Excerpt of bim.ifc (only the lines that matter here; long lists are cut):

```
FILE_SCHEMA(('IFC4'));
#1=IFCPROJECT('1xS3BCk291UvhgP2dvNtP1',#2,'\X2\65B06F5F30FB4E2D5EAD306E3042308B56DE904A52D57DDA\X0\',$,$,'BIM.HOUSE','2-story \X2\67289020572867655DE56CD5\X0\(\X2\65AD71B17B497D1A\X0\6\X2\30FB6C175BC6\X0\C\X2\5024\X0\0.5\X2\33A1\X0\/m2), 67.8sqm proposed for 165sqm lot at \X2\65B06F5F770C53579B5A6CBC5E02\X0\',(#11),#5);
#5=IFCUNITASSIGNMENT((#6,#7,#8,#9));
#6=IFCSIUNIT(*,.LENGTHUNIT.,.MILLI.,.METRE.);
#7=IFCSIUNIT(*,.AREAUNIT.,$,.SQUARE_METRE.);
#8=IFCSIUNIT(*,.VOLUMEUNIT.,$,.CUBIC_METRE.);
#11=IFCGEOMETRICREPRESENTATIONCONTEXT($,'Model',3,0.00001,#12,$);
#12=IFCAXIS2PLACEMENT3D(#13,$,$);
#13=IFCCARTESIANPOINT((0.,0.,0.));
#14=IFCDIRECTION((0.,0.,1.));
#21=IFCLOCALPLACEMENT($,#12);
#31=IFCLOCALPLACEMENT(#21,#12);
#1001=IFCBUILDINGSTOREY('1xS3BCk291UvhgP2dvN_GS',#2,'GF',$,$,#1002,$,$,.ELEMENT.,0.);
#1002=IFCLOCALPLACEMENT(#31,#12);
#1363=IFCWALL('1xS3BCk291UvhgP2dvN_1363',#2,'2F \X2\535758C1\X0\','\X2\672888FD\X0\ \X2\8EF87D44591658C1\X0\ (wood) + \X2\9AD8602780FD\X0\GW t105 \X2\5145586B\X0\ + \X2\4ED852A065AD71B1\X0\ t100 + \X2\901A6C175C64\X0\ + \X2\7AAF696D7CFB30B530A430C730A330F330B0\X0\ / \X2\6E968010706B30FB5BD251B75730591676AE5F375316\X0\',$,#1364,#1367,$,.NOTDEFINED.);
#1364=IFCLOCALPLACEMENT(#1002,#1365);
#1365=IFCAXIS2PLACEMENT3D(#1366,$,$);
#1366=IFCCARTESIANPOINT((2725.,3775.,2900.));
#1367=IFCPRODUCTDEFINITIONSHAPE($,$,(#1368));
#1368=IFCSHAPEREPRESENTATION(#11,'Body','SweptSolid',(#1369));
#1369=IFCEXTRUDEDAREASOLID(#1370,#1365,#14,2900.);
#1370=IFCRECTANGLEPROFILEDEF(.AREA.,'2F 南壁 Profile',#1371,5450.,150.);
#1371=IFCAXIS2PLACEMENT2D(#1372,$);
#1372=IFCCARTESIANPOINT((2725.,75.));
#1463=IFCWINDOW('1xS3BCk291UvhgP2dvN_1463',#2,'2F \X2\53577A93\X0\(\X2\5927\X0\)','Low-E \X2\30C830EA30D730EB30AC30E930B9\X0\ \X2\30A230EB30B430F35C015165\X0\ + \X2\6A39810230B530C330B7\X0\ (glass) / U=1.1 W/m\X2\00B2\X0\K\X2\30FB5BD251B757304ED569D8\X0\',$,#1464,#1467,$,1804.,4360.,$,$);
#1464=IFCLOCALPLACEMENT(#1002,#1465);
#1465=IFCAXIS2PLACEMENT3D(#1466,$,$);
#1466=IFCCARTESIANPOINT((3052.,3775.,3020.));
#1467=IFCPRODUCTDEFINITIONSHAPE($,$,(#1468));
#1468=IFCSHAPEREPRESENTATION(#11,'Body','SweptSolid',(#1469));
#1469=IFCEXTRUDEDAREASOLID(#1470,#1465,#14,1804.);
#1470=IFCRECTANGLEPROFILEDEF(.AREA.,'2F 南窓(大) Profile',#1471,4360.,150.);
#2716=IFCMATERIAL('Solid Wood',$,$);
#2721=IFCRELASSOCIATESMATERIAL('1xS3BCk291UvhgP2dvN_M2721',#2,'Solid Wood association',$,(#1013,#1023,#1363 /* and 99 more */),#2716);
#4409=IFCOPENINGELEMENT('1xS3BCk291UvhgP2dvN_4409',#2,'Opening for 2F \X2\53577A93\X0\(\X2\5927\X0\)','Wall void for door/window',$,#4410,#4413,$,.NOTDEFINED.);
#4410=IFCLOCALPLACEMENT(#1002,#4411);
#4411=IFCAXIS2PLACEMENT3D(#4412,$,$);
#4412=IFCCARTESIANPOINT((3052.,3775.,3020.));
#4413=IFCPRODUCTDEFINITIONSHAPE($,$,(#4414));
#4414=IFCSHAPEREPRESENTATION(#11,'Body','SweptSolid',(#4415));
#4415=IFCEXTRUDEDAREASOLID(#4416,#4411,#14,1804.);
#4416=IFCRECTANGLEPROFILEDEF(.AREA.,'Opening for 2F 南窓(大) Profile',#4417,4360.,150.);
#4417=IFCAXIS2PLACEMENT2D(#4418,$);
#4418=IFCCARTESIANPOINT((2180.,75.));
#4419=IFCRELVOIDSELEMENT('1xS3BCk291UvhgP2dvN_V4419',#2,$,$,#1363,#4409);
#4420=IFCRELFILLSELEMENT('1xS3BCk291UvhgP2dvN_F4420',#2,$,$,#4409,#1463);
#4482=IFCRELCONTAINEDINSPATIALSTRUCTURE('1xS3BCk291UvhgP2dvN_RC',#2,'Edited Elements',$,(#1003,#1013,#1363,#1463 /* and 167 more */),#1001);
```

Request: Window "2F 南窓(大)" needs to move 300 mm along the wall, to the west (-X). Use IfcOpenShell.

```python
import ifcopenshell
import ifcopenshell.api.geometry
import ifcopenshell.util.placement
import ifcopenshell.util.unit

model = ifcopenshell.open("bim.ifc")
unit_scale = ifcopenshell.util.unit.calculate_unit_scale(model)

window = model.by_id(1463)
opening = window.FillsVoids[0].RelatingOpeningElement
wall = opening.VoidsElements[0].RelatingBuildingElement

wall_matrix = ifcopenshell.util.placement.get_local_placement(wall.ObjectPlacement)
shift = wall_matrix[:3, 0] * -0.3 / unit_scale
before = ifcopenshell.util.placement.get_local_placement(window.ObjectPlacement)[:3, 3].copy()

# The window is not placed relative to its opening, so move both.
for product in (opening, window):
    matrix = ifcopenshell.util.placement.get_local_placement(product.ObjectPlacement)
    matrix[:3, 3] += shift
    ifcopenshell.api.geometry.edit_object_placement(model, product=product, matrix=matrix, is_si=False)

after = ifcopenshell.util.placement.get_local_placement(window.ObjectPlacement)[:3, 3]
print("window moved by", (after - before).round(3) + 0.0)

model.write("bim_v2.ifc")
```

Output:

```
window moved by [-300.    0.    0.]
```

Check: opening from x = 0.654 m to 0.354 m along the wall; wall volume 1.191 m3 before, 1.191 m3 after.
